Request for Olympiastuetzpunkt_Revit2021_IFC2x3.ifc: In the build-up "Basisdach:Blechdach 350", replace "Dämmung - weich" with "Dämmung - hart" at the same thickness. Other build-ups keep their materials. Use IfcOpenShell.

First a look at what the model holds.

```python
import ifcopenshell
import ifcopenshell.util.element

model = ifcopenshell.open("Olympiastuetzpunkt_Revit2021_IFC2x3.ifc")
print(model.schema)
for layer_set in model.by_type("IfcMaterialLayerSet"):
    if layer_set.LayerSetName == "Basisdach:Blechdach 350":
        for layer in layer_set.MaterialLayers:
            print(layer.id(), layer.Material and layer.Material.Name, layer.LayerThickness, sep=" | ")
        print(len(ifcopenshell.util.element.get_elements_by_material(model, layer_set)), "elements and types use it")
print(sorted(m.Name for m in model.by_type("IfcMaterial") if m.Name)[:60])
```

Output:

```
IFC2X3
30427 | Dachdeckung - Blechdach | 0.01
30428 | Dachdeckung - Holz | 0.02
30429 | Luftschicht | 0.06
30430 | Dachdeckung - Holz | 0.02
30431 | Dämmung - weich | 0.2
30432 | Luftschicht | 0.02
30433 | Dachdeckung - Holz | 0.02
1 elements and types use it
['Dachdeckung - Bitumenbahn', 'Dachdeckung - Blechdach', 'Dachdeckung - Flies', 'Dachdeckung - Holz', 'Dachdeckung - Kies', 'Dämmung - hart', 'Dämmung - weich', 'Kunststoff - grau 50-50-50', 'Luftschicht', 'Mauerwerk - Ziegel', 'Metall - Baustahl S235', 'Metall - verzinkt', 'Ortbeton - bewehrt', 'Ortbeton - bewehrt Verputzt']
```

```python
import ifcopenshell
import ifcopenshell.api.material

model = ifcopenshell.open("Olympiastuetzpunkt_Revit2021_IFC2x3.ifc")

layer_set = next(s for s in model.by_type("IfcMaterialLayerSet") if s.LayerSetName == "Basisdach:Blechdach 350")
layer = next(l for l in layer_set.MaterialLayers if l.Material and l.Material.Name == "Dämmung - weich")
material = next(m for m in model.by_type("IfcMaterial") if m.Name == "Dämmung - hart")

# Point this one layer at the other material; renaming the old one would change it everywhere.
ifcopenshell.api.material.edit_layer(model, layer=layer, attributes={}, material=material)

print([l.Material.Name if l.Material else None for l in layer_set.MaterialLayers])

model.write("Olympiastuetzpunkt_Revit2021_IFC2x3_rev.ifc")
```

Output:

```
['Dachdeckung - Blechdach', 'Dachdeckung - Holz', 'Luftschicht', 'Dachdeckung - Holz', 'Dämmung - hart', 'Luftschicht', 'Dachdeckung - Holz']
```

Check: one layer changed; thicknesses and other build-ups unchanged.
